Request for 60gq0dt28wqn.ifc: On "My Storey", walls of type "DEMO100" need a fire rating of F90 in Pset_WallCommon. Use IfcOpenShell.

First a look at what the model holds.

```python
import ifcopenshell
import ifcopenshell.util.element

model = ifcopenshell.open("60gq0dt28wqn.ifc")
print(model.schema)
storey = next(s for s in model.by_type("IfcBuildingStorey") if s.Name == "My Storey")
walls = [e for e in ifcopenshell.util.element.get_decomposition(storey) if e.is_a("IfcWall")]
seen = {}
for e in walls:
    element_type = ifcopenshell.util.element.get_type(e)
    key = (element_type.Name if element_type != e and element_type else None, ifcopenshell.util.element.get_pset(e, "Pset_WallCommon", "FireRating"))
    seen[key] = seen.get(key, 0) + 1
for (name, value), count in sorted(seen.items(), key=str):
    print(count, "x", name, "|", value)
```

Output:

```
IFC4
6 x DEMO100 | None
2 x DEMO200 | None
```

```python
import ifcopenshell
import ifcopenshell.api.pset
import ifcopenshell.util.element

model = ifcopenshell.open("60gq0dt28wqn.ifc")

storey = next(s for s in model.by_type("IfcBuildingStorey") if s.Name == "My Storey")
walls = [e for e in ifcopenshell.util.element.get_decomposition(storey) if e.is_a("IfcWall")]

count = 0
for e in walls:
    element_type = ifcopenshell.util.element.get_type(e)
    if element_type in (None, e) or element_type.Name != "DEMO100":
        continue
    # add_pset returns the element's existing set when there is one.
    pset = ifcopenshell.api.pset.add_pset(model, product=e, name="Pset_WallCommon")
    ifcopenshell.api.pset.edit_pset(model, pset=pset, properties={"FireRating": "F90"})
    count += 1

print(count, "walls updated")

model.write("60gq0dt28wqn-out.ifc")
```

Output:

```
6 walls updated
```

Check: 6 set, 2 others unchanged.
